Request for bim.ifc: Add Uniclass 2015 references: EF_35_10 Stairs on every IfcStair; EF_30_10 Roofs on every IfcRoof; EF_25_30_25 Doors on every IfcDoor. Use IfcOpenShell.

First a look at what the model holds.

```python
import ifcopenshell

model = ifcopenshell.open("bim.ifc")
print(model.schema)
print("classifications:", [c.Name for c in model.by_type("IfcClassification")])
for ifc_class in ("IfcDoor", "IfcRoof", "IfcStair", "IfcWall", "IfcWindow"):
    print(ifc_class, len(model.by_type(ifc_class)))
```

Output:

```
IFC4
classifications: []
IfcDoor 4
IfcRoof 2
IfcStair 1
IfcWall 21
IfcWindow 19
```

```python
import ifcopenshell
import ifcopenshell.api.classification

model = ifcopenshell.open("bim.ifc")

system = ifcopenshell.api.classification.add_classification(model, classification="Uniclass 2015")

codes = {
    "IfcStair": ("EF_35_10", "Stairs"),
    "IfcRoof": ("EF_30_10", "Roofs"),
    "IfcDoor": ("EF_25_30_25", "Doors"),
}
for ifc_class, (code, name) in codes.items():
    products = model.by_type(ifc_class)
    ifcopenshell.api.classification.add_reference(
        model, products=products, classification=system, identification=code, name=name
    )
    print(code, len(products))

model.write("bim_v2.ifc")
```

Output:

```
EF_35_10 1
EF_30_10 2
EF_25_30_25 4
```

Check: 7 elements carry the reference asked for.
